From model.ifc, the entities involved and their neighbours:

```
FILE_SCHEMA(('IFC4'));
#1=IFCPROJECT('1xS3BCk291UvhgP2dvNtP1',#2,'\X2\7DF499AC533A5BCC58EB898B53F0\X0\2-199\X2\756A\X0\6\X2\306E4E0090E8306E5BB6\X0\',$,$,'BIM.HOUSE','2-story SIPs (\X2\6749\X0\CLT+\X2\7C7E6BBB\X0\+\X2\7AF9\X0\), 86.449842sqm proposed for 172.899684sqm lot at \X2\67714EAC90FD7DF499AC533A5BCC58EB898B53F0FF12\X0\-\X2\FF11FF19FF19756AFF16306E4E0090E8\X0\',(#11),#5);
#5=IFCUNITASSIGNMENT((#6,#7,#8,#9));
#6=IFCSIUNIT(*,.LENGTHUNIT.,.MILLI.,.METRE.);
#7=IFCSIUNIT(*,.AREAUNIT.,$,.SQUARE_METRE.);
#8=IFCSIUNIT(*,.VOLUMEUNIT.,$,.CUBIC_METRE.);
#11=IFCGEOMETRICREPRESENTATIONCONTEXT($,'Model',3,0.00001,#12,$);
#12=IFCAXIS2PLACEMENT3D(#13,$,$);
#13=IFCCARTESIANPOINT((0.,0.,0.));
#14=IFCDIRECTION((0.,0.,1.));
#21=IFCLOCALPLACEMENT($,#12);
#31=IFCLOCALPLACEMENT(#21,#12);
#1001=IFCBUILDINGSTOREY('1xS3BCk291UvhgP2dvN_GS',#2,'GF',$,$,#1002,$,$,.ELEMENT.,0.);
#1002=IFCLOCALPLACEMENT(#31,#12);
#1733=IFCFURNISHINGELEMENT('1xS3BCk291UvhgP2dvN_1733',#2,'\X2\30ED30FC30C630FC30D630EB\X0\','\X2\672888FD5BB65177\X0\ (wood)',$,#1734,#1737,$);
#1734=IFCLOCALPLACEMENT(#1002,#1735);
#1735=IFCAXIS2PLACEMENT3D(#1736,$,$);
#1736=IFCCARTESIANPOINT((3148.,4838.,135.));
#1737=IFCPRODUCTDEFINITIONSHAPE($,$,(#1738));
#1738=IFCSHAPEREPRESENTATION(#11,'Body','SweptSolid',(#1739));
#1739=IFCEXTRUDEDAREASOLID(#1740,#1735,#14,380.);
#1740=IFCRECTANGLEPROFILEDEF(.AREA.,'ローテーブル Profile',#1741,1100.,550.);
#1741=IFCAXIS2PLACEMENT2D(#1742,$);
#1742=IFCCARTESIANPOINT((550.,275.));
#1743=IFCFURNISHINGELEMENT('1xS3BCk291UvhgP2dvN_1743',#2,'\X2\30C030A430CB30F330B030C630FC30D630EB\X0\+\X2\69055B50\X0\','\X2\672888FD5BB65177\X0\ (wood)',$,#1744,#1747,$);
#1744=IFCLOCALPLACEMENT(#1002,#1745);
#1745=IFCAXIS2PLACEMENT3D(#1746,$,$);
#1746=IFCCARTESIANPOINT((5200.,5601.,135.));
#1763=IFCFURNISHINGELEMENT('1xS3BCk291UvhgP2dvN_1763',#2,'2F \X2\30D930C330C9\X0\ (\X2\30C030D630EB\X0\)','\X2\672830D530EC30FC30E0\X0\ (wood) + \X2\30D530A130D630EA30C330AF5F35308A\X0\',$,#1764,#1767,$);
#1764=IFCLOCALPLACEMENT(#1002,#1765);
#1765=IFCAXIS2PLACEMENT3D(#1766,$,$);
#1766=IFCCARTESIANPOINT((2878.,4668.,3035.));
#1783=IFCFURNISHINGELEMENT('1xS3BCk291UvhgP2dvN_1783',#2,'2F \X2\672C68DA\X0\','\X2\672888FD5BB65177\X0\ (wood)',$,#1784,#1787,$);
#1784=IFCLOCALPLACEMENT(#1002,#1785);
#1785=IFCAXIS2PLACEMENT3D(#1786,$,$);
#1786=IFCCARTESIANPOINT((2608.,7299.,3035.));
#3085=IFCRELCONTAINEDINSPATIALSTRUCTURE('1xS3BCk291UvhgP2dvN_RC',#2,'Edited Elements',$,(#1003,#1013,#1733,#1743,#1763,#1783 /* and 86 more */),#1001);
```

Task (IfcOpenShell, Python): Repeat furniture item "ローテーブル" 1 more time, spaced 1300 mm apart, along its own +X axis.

```python
import ifcopenshell
import ifcopenshell.api.geometry
import ifcopenshell.api.root
import ifcopenshell.util.element
import ifcopenshell.util.placement

model = ifcopenshell.open("model.ifc")


def reuse_history(source, copy):
    """copy_class also copies each property set's owner history, people and application; keep the originals."""
    for rel in copy.IsDefinedBy:
        if rel.is_a("IfcRelDefinesByProperties") and (history := rel.RelatingPropertyDefinition.OwnerHistory):
            rel.RelatingPropertyDefinition.OwnerHistory = source.OwnerHistory
            ifcopenshell.util.element.remove_deep2(model, history)


source = model.by_guid("1xS3BCk291UvhgP2dvN_1733")
base = ifcopenshell.util.placement.get_local_placement(source.ObjectPlacement)
step = base[:3, 0] * 1300.0

for i in range(1, 2):
    copy = ifcopenshell.api.root.copy_class(model, product=source)
    copy.Representation = ifcopenshell.util.element.copy_deep(
        model, source.Representation, exclude=["IfcGeometricRepresentationContext", "IfcRepresentationMap"]
    )
    reuse_history(source, copy)
    matrix = base.copy()
    matrix[:3, 3] += i * step
    print("added at", matrix[:3, 3].round(3) + 0.0)
    ifcopenshell.api.geometry.edit_object_placement(model, product=copy, matrix=matrix, is_si=False)

model.write("model_rev.ifc")
```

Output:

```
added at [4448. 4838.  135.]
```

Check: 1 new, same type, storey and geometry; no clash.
